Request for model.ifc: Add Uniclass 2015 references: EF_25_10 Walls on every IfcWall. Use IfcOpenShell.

First a look at what the model holds.

```python
import ifcopenshell

model = ifcopenshell.open("model.ifc")
print(model.schema)
print("classifications:", [c.Name for c in model.by_type("IfcClassification")])
for ifc_class in ("IfcDoor", "IfcRoof", "IfcStair", "IfcWall", "IfcWindow"):
    print(ifc_class, len(model.by_type(ifc_class)))
```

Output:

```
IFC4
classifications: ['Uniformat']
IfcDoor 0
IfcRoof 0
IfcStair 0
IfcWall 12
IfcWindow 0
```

```python
import ifcopenshell
import ifcopenshell.api.classification

model = ifcopenshell.open("model.ifc")

system = ifcopenshell.api.classification.add_classification(model, classification="Uniclass 2015")

codes = {
    "IfcWall": ("EF_25_10", "Walls"),
}
for ifc_class, (code, name) in codes.items():
    products = model.by_type(ifc_class)
    ifcopenshell.api.classification.add_reference(
        model, products=products, classification=system, identification=code, name=name
    )
    print(code, len(products))

model.write("model_rev.ifc")
```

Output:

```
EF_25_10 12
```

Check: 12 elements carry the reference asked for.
